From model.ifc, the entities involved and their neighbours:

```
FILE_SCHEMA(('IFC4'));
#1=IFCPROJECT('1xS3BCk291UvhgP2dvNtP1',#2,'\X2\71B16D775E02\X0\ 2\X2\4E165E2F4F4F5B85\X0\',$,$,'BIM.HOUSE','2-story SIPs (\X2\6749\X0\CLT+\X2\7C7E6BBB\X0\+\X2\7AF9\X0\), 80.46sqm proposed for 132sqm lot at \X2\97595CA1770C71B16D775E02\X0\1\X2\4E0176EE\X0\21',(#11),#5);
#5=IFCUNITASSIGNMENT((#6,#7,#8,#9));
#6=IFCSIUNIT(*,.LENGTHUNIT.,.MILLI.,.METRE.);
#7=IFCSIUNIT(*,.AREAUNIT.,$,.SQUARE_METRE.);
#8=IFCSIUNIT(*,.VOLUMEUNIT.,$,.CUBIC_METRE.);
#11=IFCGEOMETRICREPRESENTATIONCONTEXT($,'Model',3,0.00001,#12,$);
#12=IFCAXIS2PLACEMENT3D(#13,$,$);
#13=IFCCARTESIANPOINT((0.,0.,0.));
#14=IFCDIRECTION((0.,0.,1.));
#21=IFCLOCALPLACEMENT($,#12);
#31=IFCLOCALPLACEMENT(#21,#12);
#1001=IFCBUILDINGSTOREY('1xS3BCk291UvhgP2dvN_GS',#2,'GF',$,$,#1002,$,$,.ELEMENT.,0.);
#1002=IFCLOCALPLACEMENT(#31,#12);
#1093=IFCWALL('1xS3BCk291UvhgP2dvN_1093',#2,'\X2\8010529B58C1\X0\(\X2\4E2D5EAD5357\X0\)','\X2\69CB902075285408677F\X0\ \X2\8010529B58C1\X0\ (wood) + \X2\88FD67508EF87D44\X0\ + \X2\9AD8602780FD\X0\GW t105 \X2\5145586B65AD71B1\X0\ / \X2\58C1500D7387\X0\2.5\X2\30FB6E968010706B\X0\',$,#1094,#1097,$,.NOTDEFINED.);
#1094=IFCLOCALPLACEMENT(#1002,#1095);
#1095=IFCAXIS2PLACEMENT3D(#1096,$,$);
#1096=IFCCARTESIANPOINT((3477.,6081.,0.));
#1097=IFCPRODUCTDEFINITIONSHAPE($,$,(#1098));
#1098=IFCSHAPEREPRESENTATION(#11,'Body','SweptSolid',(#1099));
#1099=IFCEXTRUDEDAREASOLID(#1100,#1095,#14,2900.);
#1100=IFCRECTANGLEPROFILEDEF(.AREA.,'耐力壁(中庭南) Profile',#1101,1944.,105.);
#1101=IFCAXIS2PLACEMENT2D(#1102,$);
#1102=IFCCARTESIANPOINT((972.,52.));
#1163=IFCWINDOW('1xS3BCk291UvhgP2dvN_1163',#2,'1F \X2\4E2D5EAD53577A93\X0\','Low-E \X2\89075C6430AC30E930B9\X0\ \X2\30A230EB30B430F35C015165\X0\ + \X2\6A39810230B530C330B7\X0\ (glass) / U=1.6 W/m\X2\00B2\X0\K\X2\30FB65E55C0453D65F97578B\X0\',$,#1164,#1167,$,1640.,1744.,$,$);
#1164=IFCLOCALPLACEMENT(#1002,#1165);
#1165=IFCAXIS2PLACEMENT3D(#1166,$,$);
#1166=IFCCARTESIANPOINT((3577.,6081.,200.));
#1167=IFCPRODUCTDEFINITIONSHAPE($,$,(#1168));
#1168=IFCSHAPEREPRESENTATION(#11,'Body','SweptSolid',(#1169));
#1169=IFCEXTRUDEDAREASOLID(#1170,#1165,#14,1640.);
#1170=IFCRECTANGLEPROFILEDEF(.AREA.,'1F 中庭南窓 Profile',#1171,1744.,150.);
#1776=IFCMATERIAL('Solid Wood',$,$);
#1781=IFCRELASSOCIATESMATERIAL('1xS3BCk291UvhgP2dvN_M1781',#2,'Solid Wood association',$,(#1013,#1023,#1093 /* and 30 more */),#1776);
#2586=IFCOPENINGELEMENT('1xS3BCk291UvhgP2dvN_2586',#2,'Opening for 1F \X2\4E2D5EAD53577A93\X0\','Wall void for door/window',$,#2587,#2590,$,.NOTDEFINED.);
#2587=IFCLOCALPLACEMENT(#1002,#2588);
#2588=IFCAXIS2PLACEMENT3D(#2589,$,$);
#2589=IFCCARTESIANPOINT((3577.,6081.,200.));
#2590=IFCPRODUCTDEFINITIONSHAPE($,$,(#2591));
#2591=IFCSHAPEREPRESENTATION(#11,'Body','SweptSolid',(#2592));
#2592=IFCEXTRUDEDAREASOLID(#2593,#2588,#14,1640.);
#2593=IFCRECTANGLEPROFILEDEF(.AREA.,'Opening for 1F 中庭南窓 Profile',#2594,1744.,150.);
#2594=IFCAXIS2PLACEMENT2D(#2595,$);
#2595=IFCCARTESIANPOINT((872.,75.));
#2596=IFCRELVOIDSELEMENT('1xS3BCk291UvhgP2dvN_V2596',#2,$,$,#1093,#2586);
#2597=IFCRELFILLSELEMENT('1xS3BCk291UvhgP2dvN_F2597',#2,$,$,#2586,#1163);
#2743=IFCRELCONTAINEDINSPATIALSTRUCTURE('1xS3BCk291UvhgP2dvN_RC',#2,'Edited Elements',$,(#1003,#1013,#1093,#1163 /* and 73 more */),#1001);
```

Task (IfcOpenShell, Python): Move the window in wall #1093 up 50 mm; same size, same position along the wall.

```python
import numpy as np
import ifcopenshell
import ifcopenshell.api.geometry
import ifcopenshell.util.placement
import ifcopenshell.util.unit

model = ifcopenshell.open("model.ifc")
unit_scale = ifcopenshell.util.unit.calculate_unit_scale(model)

window = model.by_guid("1xS3BCk291UvhgP2dvN_1163")
opening = window.FillsVoids[0].RelatingOpeningElement
dz = 0.05 / unit_scale

shift = np.array([0.0, 0.0, dz])
# The window is not placed relative to its opening, so move both.
for product in (opening, window):
    matrix = ifcopenshell.util.placement.get_local_placement(product.ObjectPlacement)
    matrix[:3, 3] += shift
    ifcopenshell.api.geometry.edit_object_placement(model, product=product, matrix=matrix, is_si=False)

print(f"moved by {dz * unit_scale:+.3f} m")

model.write("model_v2.ifc")
```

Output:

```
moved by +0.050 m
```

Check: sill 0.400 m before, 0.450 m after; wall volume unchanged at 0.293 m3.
